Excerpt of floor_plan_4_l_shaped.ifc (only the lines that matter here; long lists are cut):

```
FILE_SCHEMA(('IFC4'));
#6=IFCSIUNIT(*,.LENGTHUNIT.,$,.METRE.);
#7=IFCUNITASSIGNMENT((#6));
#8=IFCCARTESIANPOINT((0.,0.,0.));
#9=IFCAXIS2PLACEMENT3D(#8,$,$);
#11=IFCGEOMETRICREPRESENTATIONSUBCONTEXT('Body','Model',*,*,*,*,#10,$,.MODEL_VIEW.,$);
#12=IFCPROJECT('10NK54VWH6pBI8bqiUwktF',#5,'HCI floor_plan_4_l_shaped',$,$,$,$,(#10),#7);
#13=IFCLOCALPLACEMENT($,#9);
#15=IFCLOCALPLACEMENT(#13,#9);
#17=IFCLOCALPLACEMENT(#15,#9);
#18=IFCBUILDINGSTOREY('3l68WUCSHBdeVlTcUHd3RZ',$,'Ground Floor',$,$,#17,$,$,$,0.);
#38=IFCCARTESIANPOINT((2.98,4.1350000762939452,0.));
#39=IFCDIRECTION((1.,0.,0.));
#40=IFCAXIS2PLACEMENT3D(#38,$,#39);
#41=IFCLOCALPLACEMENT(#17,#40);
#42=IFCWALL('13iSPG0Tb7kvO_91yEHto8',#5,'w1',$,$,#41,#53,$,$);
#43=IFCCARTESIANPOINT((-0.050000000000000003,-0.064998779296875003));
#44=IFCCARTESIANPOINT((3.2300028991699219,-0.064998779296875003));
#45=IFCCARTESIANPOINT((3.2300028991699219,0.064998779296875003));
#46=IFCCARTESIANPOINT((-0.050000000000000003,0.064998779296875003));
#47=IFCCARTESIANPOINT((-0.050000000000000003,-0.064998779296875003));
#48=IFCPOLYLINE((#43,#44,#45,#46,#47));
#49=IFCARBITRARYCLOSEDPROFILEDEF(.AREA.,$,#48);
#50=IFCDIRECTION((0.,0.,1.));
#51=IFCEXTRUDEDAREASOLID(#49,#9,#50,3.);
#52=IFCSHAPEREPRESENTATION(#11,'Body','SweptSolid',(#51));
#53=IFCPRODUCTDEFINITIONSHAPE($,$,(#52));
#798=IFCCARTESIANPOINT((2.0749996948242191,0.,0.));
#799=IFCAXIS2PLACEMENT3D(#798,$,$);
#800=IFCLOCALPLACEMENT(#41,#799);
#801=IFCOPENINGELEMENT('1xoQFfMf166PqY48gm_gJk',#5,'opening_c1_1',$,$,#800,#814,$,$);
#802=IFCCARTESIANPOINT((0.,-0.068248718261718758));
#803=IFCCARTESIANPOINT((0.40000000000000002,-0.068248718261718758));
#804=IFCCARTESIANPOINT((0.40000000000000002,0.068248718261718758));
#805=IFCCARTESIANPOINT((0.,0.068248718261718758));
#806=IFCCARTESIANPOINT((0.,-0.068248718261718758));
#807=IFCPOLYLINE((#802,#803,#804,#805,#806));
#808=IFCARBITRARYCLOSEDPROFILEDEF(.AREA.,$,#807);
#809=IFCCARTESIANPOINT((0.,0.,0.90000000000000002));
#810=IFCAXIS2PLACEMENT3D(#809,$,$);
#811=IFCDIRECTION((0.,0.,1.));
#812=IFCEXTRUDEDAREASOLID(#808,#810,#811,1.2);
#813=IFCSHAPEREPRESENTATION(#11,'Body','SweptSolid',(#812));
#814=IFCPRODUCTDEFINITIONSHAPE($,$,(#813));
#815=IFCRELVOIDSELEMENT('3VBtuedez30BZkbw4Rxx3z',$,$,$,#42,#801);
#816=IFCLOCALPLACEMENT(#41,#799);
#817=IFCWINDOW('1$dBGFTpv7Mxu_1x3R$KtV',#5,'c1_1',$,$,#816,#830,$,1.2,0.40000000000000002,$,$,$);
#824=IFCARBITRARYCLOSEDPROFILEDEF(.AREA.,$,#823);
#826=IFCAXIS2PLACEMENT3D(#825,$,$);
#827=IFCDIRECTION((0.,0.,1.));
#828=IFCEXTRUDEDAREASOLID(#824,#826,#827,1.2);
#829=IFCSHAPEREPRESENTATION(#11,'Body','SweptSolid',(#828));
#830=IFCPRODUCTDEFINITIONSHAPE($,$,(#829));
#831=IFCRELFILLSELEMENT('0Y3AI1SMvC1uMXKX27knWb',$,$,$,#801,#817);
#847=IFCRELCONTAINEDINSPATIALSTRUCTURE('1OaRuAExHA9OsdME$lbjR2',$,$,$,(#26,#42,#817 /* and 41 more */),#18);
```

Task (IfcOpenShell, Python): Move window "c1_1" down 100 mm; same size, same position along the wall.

```python
import numpy as np
import ifcopenshell
import ifcopenshell.api.geometry
import ifcopenshell.util.placement
import ifcopenshell.util.unit

model = ifcopenshell.open("floor_plan_4_l_shaped.ifc")
unit_scale = ifcopenshell.util.unit.calculate_unit_scale(model)

window = model.by_guid("1$dBGFTpv7Mxu_1x3R$KtV")
opening = window.FillsVoids[0].RelatingOpeningElement
dz = -0.1 / unit_scale

shift = np.array([0.0, 0.0, dz])
# The window is not placed relative to its opening, so move both.
for product in (opening, window):
    matrix = ifcopenshell.util.placement.get_local_placement(product.ObjectPlacement)
    matrix[:3, 3] += shift
    ifcopenshell.api.geometry.edit_object_placement(model, product=product, matrix=matrix, is_si=False)

print(f"moved by {dz * unit_scale:+.3f} m")

model.write("floor_plan_4_l_shaped_updated.ifc")
```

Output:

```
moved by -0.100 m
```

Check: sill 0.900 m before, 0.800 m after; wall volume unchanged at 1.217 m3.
